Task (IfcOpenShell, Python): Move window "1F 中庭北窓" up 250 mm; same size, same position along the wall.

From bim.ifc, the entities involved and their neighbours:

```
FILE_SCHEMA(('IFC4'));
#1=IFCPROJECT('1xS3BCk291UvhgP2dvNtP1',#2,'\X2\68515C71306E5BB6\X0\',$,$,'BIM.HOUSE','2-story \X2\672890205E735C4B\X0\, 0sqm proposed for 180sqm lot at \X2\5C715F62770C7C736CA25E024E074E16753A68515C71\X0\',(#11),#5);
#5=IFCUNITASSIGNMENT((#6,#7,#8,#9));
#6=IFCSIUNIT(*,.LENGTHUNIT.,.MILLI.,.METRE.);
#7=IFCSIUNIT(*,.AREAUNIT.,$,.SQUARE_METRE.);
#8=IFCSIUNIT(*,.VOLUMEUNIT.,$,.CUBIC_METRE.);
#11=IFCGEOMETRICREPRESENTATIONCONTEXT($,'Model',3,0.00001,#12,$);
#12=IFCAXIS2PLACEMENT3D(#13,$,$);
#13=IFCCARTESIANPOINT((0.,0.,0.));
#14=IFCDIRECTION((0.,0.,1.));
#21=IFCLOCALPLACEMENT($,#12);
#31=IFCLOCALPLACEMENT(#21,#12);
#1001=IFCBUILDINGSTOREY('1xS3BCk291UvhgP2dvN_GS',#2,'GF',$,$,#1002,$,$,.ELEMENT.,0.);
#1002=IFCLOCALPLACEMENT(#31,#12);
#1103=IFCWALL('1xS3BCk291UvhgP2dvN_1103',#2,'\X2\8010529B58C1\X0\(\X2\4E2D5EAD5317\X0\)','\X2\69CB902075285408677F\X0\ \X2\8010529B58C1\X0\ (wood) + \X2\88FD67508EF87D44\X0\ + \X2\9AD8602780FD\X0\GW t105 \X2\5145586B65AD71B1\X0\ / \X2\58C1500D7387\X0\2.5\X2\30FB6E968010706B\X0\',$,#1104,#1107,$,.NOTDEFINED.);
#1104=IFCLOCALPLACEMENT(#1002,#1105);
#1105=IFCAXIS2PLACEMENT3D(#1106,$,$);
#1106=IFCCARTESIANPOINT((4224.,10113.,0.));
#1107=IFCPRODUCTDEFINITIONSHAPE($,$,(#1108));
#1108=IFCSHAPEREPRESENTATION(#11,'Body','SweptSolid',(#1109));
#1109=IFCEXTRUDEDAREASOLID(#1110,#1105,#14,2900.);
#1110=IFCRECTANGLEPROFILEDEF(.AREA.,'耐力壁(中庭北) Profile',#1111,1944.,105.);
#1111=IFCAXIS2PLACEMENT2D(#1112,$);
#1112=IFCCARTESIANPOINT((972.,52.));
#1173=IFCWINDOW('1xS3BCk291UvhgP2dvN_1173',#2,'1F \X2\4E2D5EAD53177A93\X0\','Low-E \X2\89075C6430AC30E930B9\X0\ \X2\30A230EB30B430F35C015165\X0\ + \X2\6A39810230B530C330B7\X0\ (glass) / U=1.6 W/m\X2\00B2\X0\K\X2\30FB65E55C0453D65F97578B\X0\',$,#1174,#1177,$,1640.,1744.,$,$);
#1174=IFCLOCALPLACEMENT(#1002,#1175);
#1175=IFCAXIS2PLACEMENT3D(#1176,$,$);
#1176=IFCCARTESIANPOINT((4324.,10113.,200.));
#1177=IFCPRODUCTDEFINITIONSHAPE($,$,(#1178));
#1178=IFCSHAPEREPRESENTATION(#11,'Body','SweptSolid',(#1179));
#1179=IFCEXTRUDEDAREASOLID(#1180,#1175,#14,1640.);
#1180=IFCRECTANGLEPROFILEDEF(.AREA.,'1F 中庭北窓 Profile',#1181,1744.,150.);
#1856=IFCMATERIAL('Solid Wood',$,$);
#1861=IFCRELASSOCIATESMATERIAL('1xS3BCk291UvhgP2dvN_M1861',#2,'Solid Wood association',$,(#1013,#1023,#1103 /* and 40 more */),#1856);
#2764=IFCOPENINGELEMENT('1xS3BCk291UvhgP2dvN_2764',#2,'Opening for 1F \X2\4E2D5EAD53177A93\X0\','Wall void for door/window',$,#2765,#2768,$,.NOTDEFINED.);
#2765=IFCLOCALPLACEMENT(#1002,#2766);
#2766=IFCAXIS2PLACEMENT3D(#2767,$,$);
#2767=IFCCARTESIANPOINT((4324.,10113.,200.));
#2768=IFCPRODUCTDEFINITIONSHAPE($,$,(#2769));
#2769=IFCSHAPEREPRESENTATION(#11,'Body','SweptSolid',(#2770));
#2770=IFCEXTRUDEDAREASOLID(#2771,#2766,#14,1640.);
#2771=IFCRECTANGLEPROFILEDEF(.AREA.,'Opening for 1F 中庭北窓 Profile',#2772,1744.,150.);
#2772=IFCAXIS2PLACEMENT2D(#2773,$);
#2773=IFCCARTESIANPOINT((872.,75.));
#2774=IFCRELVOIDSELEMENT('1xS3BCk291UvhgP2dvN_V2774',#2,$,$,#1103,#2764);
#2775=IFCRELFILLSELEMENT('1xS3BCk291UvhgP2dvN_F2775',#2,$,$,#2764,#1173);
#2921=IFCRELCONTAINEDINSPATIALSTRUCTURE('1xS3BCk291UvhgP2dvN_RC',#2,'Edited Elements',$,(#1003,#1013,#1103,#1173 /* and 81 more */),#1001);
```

```python
import numpy as np
import ifcopenshell
import ifcopenshell.api.geometry
import ifcopenshell.util.placement
import ifcopenshell.util.unit

model = ifcopenshell.open("bim.ifc")
unit_scale = ifcopenshell.util.unit.calculate_unit_scale(model)

window = model.by_guid("1xS3BCk291UvhgP2dvN_1173")
opening = window.FillsVoids[0].RelatingOpeningElement
dz = 250.0

shift = np.array([0.0, 0.0, dz])
# The window is not placed relative to its opening, so move both.
for product in (opening, window):
    matrix = ifcopenshell.util.placement.get_local_placement(product.ObjectPlacement)
    matrix[:3, 3] += shift
    ifcopenshell.api.geometry.edit_object_placement(model, product=product, matrix=matrix, is_si=False)

print(f"moved by {dz * unit_scale:+.3f} m")

model.write("bim_rev.ifc")
```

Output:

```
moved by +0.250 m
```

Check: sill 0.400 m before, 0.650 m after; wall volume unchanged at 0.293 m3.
